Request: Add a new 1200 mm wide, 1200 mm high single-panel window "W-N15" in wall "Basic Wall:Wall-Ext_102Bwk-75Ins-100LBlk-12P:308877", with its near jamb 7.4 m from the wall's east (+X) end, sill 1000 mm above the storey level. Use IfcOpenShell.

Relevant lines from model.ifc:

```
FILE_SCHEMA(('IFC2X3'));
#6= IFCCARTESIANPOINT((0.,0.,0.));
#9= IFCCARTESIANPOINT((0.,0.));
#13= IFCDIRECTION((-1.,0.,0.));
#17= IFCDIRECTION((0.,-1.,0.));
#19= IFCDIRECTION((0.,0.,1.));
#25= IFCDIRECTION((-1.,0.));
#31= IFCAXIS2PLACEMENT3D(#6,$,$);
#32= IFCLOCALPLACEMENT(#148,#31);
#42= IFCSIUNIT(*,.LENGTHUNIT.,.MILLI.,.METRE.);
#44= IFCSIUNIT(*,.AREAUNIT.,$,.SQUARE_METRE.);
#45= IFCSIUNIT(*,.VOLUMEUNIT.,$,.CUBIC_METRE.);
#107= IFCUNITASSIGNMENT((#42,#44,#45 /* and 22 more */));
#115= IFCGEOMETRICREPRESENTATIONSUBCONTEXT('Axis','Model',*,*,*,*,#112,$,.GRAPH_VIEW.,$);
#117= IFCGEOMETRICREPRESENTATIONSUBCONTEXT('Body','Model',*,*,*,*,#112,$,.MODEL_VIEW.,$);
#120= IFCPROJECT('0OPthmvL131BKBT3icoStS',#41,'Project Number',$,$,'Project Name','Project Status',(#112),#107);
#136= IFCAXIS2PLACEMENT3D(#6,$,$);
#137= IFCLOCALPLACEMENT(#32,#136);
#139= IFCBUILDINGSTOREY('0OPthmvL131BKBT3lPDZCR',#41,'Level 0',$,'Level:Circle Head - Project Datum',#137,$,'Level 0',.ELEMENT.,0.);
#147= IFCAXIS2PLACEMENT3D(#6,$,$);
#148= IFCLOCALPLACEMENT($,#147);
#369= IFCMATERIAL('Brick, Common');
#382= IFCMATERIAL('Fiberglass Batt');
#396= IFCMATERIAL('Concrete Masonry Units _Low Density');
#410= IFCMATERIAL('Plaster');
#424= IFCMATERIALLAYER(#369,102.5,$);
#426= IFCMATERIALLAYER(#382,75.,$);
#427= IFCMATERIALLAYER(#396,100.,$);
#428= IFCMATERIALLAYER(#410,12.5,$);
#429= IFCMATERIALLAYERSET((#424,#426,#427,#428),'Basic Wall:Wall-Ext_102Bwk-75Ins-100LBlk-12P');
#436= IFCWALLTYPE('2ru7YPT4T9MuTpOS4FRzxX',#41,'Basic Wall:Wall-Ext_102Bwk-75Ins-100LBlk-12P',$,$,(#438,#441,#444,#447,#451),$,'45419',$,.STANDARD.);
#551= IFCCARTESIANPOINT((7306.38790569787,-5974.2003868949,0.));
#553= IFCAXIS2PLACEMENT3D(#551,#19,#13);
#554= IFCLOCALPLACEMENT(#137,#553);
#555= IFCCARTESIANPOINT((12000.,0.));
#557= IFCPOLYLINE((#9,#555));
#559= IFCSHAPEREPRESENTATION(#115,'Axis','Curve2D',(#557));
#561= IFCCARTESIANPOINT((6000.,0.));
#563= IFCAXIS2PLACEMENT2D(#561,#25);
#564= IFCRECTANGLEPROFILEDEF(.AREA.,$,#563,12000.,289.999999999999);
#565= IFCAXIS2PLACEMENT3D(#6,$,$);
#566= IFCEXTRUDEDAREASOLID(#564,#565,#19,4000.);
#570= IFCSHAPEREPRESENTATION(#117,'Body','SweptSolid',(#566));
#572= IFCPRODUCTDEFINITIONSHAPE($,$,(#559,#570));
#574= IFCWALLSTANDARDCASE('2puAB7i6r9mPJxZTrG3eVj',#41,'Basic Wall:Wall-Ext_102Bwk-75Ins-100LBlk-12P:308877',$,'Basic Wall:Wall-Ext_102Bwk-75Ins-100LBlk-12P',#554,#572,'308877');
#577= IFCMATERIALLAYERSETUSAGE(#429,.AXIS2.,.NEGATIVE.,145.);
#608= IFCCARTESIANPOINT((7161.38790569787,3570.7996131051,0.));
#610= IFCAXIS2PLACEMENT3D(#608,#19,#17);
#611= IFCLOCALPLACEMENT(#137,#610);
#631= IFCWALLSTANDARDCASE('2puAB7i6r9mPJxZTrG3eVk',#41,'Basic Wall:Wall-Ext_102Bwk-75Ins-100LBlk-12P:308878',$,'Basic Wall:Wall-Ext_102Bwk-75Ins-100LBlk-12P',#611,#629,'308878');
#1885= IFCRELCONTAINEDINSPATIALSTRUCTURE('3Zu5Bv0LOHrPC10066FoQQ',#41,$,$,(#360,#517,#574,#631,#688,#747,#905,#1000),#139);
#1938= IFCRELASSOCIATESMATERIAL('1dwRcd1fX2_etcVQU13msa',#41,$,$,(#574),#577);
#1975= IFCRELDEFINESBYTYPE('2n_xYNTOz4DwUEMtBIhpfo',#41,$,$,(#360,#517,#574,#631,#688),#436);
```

```python
import numpy as np
import ifcopenshell
import ifcopenshell.api.feature
import ifcopenshell.api.geometry
import ifcopenshell.api.root
import ifcopenshell.api.spatial
import ifcopenshell.api.type
import ifcopenshell.geom
import ifcopenshell.util.element
import ifcopenshell.util.placement
import ifcopenshell.util.representation
import ifcopenshell.util.shape
import ifcopenshell.util.unit

model = ifcopenshell.open("model.ifc")
unit_scale = ifcopenshell.util.unit.calculate_unit_scale(model)
settings = ifcopenshell.geom.settings()


def volume(element):
    """Net volume in cubic metres, openings subtracted."""
    shape = ifcopenshell.geom.create_shape(settings, element)
    return ifcopenshell.util.shape.get_volume(shape.geometry)


wall = model.by_guid("2puAB7i6r9mPJxZTrG3eVj")
storey = ifcopenshell.util.element.get_container(wall, ifc_class="IfcBuildingStorey")
context = ifcopenshell.util.representation.get_context(model, "Model", "Body", "MODEL_VIEW")
before = volume(wall)

width, height, from_end, sill = 1.2, 1.2, 7.4, 1  # metres

# The wall runs along its own X axis, and the end named is its -X end.
wall_shape = ifcopenshell.geom.create_shape(settings, wall)
x, y, z = ifcopenshell.util.shape.get_vertices(wall_shape.geometry).T
start = x.min() + from_end
face, thickness = float(y.min()), float(y.max() - y.min())
wall_matrix = ifcopenshell.util.placement.get_local_placement(wall.ObjectPlacement)
level = ifcopenshell.util.placement.get_local_placement(storey.ObjectPlacement)[2, 3]


def in_wall(x, y):
    """Placement at x, y metres in the wall's axes, at sill height."""
    matrix = wall_matrix.copy()
    matrix[:, 3] = wall_matrix @ np.array([x / unit_scale, y / unit_scale, 0.0, 1.0])
    matrix[2, 3] = level + sill / unit_scale
    return matrix


# Opening: a box that overshoots both wall faces by 50 mm.
opening = ifcopenshell.api.root.create_entity(model, ifc_class="IfcOpeningElement")
box = ifcopenshell.api.geometry.add_wall_representation(
    model, context=context, length=width, height=height, thickness=thickness + 0.1
)
ifcopenshell.api.geometry.assign_representation(model, product=opening, representation=box)
ifcopenshell.api.geometry.edit_object_placement(model, product=opening, matrix=in_wall(start, face - 0.05), is_si=False)
ifcopenshell.api.feature.add_feature(model, feature=opening, element=wall)

window = ifcopenshell.api.root.create_entity(model, ifc_class="IfcWindow", name="W-N15")
window.OverallWidth, window.OverallHeight = width / unit_scale, height / unit_scale
body = ifcopenshell.api.geometry.add_window_representation(
    model,
    context=context,
    overall_width=window.OverallWidth,
    overall_height=window.OverallHeight,
    partition_type="SINGLE_PANEL",
)
ifcopenshell.api.geometry.assign_representation(model, product=window, representation=body)
ifcopenshell.api.spatial.assign_container(model, products=[window], relating_structure=storey)
fills = ifcopenshell.api.feature.add_filling(model, opening=opening, element=window)
fills.OwnerHistory = window.OwnerHistory  # required in IFC2X3

# IFC2X3 keeps the operation on the window style.
style = ifcopenshell.api.root.create_entity(model, ifc_class="IfcWindowStyle", name="W-N15")
style.OperationType, style.ConstructionType = "SINGLE_PANEL", "NOTDEFINED"
style.ParameterTakesPrecedence = style.Sizeable = False
ifcopenshell.api.type.assign_type(model, related_objects=[window], relating_type=style)

# Centre the window in the wall's thickness.
ifcopenshell.api.geometry.edit_object_placement(model, product=window, matrix=in_wall(start, face), is_si=False)
window_shape = ifcopenshell.geom.create_shape(settings, window)
depth = ifcopenshell.util.shape.get_vertices(window_shape.geometry)[:, 1]
offset = face + thickness / 2 - (depth.min() + depth.max()) / 2
ifcopenshell.api.geometry.edit_object_placement(model, product=window, matrix=in_wall(start, offset), is_si=False)

after = volume(wall)

print(f"wall volume {before:.3f} -> {after:.3f} m3")

model.write("model_rev.ifc")
```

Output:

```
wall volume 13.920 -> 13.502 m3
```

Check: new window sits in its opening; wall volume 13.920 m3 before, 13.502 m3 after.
